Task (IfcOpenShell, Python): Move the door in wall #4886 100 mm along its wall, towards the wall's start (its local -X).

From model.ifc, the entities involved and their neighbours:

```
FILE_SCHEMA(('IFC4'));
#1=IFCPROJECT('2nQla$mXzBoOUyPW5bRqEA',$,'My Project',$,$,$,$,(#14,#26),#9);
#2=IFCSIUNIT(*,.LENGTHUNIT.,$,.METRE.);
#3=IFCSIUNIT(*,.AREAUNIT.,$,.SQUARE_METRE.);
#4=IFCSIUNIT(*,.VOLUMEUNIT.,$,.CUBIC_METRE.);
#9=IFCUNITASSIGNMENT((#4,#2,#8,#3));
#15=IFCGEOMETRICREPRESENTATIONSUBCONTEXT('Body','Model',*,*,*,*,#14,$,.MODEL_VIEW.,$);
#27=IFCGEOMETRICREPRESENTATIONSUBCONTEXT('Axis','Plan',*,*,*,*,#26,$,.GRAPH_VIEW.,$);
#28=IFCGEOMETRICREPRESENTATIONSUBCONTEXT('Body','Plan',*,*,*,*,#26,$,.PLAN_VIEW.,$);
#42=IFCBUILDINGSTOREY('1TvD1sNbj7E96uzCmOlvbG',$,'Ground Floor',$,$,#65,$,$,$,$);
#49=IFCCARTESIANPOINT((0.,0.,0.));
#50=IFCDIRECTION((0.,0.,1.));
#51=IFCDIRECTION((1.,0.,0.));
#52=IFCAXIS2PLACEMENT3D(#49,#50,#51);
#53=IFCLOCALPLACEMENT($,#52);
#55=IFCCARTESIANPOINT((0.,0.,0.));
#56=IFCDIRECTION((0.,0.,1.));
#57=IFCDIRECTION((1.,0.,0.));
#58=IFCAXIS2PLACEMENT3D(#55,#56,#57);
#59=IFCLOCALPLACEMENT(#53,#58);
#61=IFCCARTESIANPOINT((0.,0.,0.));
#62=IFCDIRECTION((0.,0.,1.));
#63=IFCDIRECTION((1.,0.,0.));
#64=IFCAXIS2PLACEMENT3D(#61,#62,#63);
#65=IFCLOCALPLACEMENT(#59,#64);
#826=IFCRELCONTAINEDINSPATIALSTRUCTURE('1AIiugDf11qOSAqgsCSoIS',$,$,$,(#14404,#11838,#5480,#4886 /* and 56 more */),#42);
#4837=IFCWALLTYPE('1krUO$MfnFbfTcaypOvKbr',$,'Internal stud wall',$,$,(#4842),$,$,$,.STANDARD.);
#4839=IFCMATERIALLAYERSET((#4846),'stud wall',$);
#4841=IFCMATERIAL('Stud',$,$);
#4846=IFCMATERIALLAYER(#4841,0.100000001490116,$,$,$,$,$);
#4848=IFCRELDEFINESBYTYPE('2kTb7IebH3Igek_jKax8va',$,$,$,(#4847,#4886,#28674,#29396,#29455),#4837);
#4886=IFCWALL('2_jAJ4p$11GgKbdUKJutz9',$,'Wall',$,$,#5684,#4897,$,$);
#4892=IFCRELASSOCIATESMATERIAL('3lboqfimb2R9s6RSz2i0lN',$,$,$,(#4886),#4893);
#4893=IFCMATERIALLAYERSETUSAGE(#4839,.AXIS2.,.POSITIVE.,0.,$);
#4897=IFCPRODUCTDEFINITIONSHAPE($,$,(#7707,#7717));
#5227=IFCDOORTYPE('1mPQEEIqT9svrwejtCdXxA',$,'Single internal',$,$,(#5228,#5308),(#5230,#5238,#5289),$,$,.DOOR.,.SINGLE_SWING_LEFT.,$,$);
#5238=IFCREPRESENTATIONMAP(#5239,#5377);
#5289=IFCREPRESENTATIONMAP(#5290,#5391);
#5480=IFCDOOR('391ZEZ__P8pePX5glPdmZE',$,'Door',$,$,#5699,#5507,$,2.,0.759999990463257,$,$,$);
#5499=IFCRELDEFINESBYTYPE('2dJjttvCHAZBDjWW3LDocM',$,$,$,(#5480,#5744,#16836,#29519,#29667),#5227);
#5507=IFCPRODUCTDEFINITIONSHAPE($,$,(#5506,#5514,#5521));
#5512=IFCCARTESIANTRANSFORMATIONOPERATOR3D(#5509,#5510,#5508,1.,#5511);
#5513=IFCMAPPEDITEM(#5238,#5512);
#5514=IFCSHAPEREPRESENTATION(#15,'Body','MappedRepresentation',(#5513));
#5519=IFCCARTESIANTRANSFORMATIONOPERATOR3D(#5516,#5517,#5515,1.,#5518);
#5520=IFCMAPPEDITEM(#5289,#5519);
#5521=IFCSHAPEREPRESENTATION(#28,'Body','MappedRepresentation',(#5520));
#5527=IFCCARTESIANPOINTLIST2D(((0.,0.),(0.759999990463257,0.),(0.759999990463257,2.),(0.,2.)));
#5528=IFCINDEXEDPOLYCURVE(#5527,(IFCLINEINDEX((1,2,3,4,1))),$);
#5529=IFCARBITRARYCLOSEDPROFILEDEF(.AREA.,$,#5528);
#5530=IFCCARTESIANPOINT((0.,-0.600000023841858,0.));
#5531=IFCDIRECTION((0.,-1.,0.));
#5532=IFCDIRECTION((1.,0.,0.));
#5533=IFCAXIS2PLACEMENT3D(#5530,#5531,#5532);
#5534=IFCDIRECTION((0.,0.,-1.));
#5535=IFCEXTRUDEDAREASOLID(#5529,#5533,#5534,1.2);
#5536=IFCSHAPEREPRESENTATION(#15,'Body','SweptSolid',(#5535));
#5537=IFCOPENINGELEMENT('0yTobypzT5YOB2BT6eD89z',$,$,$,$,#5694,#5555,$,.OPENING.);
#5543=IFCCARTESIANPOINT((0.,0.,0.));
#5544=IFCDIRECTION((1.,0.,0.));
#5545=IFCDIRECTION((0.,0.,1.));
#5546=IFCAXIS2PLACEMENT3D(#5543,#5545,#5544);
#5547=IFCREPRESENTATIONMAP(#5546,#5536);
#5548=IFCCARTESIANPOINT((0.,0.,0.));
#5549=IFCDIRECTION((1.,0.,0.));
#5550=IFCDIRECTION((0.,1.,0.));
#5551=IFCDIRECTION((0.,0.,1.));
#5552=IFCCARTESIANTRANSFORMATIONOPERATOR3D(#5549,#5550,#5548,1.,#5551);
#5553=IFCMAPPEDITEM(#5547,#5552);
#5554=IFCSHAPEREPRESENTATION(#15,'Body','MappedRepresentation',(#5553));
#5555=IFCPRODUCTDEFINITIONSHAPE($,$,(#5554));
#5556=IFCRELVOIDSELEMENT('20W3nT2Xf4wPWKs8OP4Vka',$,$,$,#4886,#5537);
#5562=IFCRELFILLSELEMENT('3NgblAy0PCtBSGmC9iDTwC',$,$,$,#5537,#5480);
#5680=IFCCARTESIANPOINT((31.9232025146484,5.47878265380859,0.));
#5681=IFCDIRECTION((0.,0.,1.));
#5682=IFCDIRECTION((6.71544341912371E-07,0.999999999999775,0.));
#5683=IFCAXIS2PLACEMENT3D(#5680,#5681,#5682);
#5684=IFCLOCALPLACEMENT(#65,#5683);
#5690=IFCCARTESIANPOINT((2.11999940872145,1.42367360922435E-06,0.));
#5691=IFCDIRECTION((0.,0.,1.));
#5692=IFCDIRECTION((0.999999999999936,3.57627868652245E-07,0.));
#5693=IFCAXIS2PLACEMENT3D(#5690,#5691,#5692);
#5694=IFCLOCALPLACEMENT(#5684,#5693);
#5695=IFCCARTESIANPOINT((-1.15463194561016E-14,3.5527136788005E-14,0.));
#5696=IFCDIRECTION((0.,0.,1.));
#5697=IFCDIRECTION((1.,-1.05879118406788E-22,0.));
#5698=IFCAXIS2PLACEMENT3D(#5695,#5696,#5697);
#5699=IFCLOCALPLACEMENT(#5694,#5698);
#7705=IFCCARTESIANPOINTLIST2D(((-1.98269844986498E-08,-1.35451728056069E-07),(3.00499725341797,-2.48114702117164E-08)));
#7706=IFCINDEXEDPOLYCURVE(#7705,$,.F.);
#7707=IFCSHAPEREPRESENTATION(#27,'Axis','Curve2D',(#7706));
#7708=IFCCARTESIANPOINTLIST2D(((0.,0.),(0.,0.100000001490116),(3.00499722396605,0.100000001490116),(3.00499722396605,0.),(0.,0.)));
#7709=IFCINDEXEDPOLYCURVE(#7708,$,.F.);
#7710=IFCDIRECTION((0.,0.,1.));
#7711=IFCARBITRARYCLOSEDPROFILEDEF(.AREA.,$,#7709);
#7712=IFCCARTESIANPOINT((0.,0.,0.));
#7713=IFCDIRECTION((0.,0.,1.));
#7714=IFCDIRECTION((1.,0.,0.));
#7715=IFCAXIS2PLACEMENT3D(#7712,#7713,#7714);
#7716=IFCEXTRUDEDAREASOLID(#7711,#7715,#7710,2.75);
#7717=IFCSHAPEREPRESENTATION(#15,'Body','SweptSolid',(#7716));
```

```python
import ifcopenshell
import ifcopenshell.api.geometry
import ifcopenshell.util.placement
import ifcopenshell.util.unit

model = ifcopenshell.open("model.ifc")
unit_scale = ifcopenshell.util.unit.calculate_unit_scale(model)

door = model.by_guid("391ZEZ__P8pePX5glPdmZE")
opening = door.FillsVoids[0].RelatingOpeningElement
wall = opening.VoidsElements[0].RelatingBuildingElement

wall_matrix = ifcopenshell.util.placement.get_local_placement(wall.ObjectPlacement)
shift = wall_matrix[:3, 0] * -0.1 / unit_scale
before = ifcopenshell.util.placement.get_local_placement(door.ObjectPlacement)[:3, 3].copy()

# The door is placed relative to its opening, so it follows when the opening moves.
matrix = ifcopenshell.util.placement.get_local_placement(opening.ObjectPlacement)
matrix[:3, 3] += shift
ifcopenshell.api.geometry.edit_object_placement(
    model, product=opening, matrix=matrix, is_si=False, should_transform_children=True
)

after = ifcopenshell.util.placement.get_local_placement(door.ObjectPlacement)[:3, 3]
print("door moved by", (after - before).round(3) + 0.0)

model.write("model_v2.ifc")
```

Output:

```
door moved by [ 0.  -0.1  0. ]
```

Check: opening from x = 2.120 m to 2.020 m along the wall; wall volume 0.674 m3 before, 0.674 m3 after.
